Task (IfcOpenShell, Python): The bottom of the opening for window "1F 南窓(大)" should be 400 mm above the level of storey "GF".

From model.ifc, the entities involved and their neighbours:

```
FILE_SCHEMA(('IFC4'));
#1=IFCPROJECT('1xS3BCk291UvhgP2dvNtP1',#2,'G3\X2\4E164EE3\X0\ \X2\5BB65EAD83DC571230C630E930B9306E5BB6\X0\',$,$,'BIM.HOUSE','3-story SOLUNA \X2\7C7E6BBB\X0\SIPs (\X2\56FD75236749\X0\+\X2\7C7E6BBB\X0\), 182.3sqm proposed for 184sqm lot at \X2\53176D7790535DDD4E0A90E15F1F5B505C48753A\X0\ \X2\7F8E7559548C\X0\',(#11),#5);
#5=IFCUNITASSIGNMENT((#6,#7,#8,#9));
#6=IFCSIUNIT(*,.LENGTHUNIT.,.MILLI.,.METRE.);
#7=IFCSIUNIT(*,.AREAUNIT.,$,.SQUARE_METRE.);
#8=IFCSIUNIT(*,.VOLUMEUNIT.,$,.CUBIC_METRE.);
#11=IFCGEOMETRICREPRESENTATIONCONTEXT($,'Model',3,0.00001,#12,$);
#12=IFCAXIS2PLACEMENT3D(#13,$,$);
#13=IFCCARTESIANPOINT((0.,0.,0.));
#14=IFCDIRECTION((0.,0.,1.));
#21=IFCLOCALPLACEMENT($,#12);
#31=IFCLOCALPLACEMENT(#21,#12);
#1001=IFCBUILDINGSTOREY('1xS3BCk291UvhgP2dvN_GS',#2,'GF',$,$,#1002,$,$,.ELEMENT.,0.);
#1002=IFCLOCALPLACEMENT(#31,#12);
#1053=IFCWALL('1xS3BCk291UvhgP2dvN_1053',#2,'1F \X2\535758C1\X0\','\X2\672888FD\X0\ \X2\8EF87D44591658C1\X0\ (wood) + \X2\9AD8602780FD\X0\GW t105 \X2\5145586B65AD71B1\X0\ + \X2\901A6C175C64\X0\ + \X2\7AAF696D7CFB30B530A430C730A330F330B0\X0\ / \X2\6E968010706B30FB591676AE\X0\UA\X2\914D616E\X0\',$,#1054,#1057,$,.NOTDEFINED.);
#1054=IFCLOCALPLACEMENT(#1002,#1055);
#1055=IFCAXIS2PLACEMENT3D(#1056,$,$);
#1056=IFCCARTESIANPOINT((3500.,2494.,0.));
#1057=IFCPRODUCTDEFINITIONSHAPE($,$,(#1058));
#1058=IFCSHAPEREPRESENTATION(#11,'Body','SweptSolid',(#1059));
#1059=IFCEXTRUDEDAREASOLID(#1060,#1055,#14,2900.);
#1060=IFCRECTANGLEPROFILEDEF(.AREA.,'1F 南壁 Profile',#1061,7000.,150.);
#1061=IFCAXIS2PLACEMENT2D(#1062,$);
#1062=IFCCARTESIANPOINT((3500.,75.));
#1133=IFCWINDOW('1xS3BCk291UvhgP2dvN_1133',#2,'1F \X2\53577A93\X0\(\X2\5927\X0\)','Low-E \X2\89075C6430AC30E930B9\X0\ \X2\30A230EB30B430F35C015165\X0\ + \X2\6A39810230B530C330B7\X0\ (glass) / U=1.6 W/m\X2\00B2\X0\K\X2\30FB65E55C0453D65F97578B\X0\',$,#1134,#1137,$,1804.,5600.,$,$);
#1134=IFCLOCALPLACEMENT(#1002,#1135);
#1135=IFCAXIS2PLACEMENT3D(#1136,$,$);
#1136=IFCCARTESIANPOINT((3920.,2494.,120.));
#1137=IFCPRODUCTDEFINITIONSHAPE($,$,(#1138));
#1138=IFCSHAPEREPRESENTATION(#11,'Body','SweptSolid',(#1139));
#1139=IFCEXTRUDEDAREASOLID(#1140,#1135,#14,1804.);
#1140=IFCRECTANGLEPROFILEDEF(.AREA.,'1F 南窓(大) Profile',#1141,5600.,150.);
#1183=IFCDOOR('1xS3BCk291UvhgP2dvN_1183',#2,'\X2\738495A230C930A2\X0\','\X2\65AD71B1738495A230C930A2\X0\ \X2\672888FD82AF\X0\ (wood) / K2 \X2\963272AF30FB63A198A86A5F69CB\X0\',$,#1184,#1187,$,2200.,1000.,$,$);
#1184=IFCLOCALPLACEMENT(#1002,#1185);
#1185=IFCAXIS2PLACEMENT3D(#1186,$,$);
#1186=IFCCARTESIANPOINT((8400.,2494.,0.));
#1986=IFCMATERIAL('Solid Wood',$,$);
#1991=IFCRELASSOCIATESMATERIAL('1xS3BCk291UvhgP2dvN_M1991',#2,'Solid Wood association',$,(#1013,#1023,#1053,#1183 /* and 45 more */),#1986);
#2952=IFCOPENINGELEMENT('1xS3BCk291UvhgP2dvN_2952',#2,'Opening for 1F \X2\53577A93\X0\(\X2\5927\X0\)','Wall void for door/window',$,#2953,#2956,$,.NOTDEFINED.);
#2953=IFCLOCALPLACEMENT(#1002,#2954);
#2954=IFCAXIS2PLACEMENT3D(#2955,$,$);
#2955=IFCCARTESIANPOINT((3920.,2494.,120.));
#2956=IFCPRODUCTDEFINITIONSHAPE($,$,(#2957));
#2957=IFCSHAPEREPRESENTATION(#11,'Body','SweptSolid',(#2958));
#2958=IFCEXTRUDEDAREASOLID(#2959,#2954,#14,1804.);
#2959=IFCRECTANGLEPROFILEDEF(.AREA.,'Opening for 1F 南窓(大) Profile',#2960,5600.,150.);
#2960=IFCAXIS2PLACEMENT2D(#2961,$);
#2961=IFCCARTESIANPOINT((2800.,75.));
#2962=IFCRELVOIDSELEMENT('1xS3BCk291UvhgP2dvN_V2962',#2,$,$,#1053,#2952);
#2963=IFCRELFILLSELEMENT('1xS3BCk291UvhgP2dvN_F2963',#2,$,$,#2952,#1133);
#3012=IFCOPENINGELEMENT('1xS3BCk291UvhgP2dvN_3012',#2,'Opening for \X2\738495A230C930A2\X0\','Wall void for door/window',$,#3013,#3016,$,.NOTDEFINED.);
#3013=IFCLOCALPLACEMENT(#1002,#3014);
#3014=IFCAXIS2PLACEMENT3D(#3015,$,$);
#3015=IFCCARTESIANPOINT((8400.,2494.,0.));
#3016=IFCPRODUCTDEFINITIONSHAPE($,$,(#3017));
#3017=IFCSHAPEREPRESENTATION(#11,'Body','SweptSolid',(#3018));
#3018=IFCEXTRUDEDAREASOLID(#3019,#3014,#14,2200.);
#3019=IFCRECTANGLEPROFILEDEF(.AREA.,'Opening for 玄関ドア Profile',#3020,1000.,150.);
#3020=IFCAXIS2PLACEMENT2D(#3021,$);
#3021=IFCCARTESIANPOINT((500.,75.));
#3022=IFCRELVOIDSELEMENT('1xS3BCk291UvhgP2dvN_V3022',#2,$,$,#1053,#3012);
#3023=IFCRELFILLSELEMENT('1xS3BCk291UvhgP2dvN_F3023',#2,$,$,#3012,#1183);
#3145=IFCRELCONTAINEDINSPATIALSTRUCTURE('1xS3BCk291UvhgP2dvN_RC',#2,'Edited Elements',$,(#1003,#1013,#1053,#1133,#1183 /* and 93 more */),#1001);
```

```python
import numpy as np
import ifcopenshell
import ifcopenshell.api.geometry
import ifcopenshell.geom
import ifcopenshell.util.element
import ifcopenshell.util.placement
import ifcopenshell.util.shape
import ifcopenshell.util.unit

model = ifcopenshell.open("model.ifc")
unit_scale = ifcopenshell.util.unit.calculate_unit_scale(model)

window = model.by_id(1133)
opening = window.FillsVoids[0].RelatingOpeningElement
storey = ifcopenshell.util.element.get_container(window, ifc_class="IfcBuildingStorey")
level = ifcopenshell.util.placement.get_local_placement(storey.ObjectPlacement)[2, 3]

# The opening's origin need not be at the sill, so measure its lowest point.
shape = ifcopenshell.geom.create_shape(ifcopenshell.geom.settings(), opening)
bottom = ifcopenshell.util.shape.get_shape_bottom_elevation(shape, shape.geometry) / unit_scale
dz = level + 400.0 - bottom

shift = np.array([0.0, 0.0, dz])
# The window is not placed relative to its opening, so move both.
for product in (opening, window):
    matrix = ifcopenshell.util.placement.get_local_placement(product.ObjectPlacement)
    matrix[:3, 3] += shift
    ifcopenshell.api.geometry.edit_object_placement(model, product=product, matrix=matrix, is_si=False)

print(f"moved by {dz * unit_scale:+.3f} m")

model.write("model-out.ifc")
```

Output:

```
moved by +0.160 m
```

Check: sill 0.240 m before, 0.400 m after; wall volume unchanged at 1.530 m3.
